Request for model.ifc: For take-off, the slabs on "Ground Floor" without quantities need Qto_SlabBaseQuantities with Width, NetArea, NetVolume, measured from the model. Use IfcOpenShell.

First a look at what the model holds.

```python
import ifcopenshell
import ifcopenshell.util.element
import ifcopenshell.util.unit

model = ifcopenshell.open("model.ifc")
print(model.schema)
for unit_type in ("LENGTHUNIT", "AREAUNIT", "VOLUMEUNIT"):
    print(unit_type, ifcopenshell.util.unit.calculate_unit_scale(model, unit_type))
storey = next(s for s in model.by_type("IfcBuildingStorey") if s.Name == "Ground Floor")
slabs = [e for e in ifcopenshell.util.element.get_decomposition(storey) if e.is_a("IfcSlab")]
for e in sorted(slabs, key=lambda e: e.id()):
    print(e.id(), e.is_a(), e.Name, list(ifcopenshell.util.element.get_psets(e, qtos_only=True)), sep=" | ")
```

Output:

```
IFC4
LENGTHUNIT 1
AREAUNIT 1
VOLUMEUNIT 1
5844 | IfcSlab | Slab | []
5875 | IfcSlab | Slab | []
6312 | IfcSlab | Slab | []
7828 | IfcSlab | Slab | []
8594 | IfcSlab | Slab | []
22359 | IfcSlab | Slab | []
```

```python
import ifcopenshell
import ifcopenshell.api.pset
import ifcopenshell.geom
import ifcopenshell.util.element
import ifcopenshell.util.shape
import ifcopenshell.util.unit

model = ifcopenshell.open("model.ifc")
unit_scale = ifcopenshell.util.unit.calculate_unit_scale(model)
area_scale = ifcopenshell.util.unit.calculate_unit_scale(model, "AREAUNIT")
volume_scale = ifcopenshell.util.unit.calculate_unit_scale(model, "VOLUMEUNIT")
settings = ifcopenshell.geom.settings()

storey = next(s for s in model.by_type("IfcBuildingStorey") if s.Name == "Ground Floor")
slabs = [e for e in ifcopenshell.util.element.get_decomposition(storey) if e.is_a("IfcSlab")]

for e in sorted(slabs, key=lambda e: e.id()):
    if ifcopenshell.util.element.get_psets(e, qtos_only=True, should_inherit=False):
        continue
    # Geometry comes back in metres, in the element's own axes.
    shape = ifcopenshell.geom.create_shape(settings, e)
    values = {
        "Width": ifcopenshell.util.shape.get_z(shape.geometry) / unit_scale,
        "NetArea": ifcopenshell.util.shape.get_footprint_area(shape.geometry) / area_scale,
        "NetVolume": ifcopenshell.util.shape.get_volume(shape.geometry) / volume_scale,
    }
    qto = ifcopenshell.api.pset.add_qto(model, product=e, name="Qto_SlabBaseQuantities")
    ifcopenshell.api.pset.edit_qto(model, qto=qto, properties=values)
    print(e.id(), {k: round(v, 3) for k, v in values.items()})

model.write("model_updated.ifc")
```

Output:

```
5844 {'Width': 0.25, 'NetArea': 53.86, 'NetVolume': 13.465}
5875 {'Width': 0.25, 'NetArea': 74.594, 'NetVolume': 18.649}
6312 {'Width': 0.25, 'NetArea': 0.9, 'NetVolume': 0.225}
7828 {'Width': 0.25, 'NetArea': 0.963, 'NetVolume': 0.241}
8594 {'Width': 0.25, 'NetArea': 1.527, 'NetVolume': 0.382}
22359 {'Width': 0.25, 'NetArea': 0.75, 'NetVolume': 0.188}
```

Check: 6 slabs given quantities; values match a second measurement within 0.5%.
